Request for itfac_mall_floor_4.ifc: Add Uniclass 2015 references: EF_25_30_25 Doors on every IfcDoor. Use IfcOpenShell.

First a look at what the model holds.

```python
import ifcopenshell

model = ifcopenshell.open("itfac_mall_floor_4.ifc")
print(model.schema)
print("classifications:", [c.Name for c in model.by_type("IfcClassification")])
for ifc_class in ("IfcDoor", "IfcRoof", "IfcStair", "IfcWall", "IfcWindow"):
    print(ifc_class, len(model.by_type(ifc_class)))
```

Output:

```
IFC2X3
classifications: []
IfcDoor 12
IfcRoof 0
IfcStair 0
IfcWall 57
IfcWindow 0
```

```python
import ifcopenshell
import ifcopenshell.api.classification

model = ifcopenshell.open("itfac_mall_floor_4.ifc")

# IFC2X3 requires Source and Edition and has no link from the project to the system.
system = model.create_entity("IfcClassification", Source="NBS", Edition="2015", Name="Uniclass 2015")

codes = {
    "IfcDoor": ("EF_25_30_25", "Doors"),
}
for ifc_class, (code, name) in codes.items():
    products = model.by_type(ifc_class)
    ifcopenshell.api.classification.add_reference(
        model, products=products, classification=system, identification=code, name=name
    )
    print(code, len(products))

model.write("itfac_mall_floor_4_rev.ifc")
```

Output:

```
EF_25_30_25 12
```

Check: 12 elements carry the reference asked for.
